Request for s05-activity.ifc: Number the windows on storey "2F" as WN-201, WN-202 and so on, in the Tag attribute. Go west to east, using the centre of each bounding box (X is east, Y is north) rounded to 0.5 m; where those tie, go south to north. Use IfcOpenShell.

First a look at what the model holds.

```python
import ifcopenshell
import ifcopenshell.util.element
import ifcopenshell.util.placement

model = ifcopenshell.open("s05-activity.ifc")
print(model.schema)
storey = next(s for s in model.by_type("IfcBuildingStorey") if s.Name == "2F")
windows = [e for e in ifcopenshell.util.element.get_decomposition(storey) if e.is_a("IfcWindow")]
for e in sorted(windows, key=lambda e: e.id()):
    origin = ifcopenshell.util.placement.get_local_placement(e.ObjectPlacement)[:3, 3]
    print(e.id(), e.Tag, e.Name, origin.round(2) + 0.0, sep=" | ")
```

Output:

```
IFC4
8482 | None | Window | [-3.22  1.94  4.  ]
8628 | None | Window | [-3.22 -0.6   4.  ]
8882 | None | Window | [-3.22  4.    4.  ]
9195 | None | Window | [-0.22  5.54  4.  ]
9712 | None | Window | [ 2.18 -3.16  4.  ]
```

```python
import ifcopenshell
import ifcopenshell.geom
import ifcopenshell.util.element
import ifcopenshell.util.shape

model = ifcopenshell.open("s05-activity.ifc")
settings = ifcopenshell.geom.settings()
settings.set("use-world-coords", True)


def centre(element):
    shape = ifcopenshell.geom.create_shape(settings, element)
    return ifcopenshell.util.shape.get_bbox_centroid(shape.geometry)


storey = next(s for s in model.by_type("IfcBuildingStorey") if s.Name == "2F")
windows = [e for e in ifcopenshell.util.element.get_decomposition(storey) if e.is_a("IfcWindow")]

# Insertion points can sit at a corner or the storey origin, so sort by the geometry (in metres).
centres = {e: centre(e) for e in windows}
windows.sort(key=lambda e: (round(centres[e][0] / 0.5), centres[e][1]))

for i, e in enumerate(windows, start=1):
    number = f"WN-2{i:02d}"
    e.Tag = number
    print(e.id(), number)

model.write("s05-activity_edited.ifc")
```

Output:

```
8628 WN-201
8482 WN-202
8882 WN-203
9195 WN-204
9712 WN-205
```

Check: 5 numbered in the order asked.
